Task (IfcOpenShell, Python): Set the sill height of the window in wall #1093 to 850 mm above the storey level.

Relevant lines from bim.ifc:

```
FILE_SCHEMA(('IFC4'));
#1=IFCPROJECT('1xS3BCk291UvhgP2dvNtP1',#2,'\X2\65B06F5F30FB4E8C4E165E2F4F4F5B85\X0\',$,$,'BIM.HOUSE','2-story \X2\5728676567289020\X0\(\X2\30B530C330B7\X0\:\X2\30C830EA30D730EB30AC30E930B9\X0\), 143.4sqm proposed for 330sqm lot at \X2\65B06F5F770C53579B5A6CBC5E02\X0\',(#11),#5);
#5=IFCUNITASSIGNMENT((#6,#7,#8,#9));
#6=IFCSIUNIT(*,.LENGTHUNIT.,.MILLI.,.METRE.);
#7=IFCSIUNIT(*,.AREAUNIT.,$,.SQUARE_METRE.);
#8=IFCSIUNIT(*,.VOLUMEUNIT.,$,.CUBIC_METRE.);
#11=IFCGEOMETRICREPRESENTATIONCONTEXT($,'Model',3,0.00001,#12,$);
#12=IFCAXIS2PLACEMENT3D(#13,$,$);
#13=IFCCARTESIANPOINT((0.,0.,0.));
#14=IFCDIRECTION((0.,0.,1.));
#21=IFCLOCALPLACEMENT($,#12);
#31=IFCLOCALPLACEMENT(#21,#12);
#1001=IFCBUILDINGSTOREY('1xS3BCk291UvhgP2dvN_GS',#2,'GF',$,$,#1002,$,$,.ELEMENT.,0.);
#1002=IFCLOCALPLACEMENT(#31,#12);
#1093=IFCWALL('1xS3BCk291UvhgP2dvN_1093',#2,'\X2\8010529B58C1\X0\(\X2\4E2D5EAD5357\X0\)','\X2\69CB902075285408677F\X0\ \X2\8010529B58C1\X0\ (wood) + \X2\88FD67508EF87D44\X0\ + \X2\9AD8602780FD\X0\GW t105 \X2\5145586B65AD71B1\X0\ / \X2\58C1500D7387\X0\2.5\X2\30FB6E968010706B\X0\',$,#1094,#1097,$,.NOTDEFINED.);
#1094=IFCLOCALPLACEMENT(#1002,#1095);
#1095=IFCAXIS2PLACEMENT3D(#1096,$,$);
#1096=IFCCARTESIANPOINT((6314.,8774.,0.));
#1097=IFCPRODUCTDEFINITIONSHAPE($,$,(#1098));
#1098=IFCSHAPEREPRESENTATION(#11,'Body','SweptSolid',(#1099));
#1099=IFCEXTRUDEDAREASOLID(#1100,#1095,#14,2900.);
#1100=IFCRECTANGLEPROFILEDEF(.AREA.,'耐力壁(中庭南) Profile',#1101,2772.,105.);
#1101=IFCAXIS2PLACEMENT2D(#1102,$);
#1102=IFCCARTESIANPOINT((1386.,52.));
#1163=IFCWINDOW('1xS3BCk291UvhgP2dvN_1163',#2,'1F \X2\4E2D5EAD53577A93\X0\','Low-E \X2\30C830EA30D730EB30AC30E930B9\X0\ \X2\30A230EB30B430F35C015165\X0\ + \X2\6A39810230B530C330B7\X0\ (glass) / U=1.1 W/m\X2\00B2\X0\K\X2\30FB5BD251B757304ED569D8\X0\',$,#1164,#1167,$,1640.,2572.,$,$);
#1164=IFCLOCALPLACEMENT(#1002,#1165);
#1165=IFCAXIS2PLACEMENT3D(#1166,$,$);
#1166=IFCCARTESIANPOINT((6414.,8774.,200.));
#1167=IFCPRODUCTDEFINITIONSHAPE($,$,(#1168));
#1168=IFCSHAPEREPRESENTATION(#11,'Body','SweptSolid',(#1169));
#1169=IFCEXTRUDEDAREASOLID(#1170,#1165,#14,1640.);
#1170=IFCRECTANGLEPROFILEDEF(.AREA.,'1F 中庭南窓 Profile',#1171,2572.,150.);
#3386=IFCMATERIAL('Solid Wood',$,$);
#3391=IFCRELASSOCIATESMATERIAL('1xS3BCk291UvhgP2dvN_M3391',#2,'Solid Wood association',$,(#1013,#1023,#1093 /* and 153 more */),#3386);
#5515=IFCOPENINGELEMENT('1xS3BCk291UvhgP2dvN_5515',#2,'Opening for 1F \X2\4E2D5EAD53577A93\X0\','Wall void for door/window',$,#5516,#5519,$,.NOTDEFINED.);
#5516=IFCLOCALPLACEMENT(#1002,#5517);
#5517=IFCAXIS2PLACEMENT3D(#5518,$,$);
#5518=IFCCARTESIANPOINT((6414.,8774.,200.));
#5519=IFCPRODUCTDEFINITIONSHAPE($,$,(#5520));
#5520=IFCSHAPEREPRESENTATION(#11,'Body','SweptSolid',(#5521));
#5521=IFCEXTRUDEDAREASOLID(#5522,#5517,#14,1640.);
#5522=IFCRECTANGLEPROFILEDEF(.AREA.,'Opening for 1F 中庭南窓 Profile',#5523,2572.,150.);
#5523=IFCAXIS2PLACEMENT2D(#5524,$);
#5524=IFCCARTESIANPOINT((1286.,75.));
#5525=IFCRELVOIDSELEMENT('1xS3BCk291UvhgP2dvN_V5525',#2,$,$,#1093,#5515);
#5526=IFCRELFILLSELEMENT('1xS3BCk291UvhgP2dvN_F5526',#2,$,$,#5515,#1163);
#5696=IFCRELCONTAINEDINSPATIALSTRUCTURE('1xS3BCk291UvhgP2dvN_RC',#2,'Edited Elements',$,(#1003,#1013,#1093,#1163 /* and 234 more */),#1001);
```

```python
import numpy as np
import ifcopenshell
import ifcopenshell.api.geometry
import ifcopenshell.geom
import ifcopenshell.util.element
import ifcopenshell.util.placement
import ifcopenshell.util.shape
import ifcopenshell.util.unit

model = ifcopenshell.open("bim.ifc")
unit_scale = ifcopenshell.util.unit.calculate_unit_scale(model)

window = model.by_id(1163)
opening = window.FillsVoids[0].RelatingOpeningElement
storey = ifcopenshell.util.element.get_container(window, ifc_class="IfcBuildingStorey")
level = ifcopenshell.util.placement.get_local_placement(storey.ObjectPlacement)[2, 3]

# The opening's origin need not be at the sill, so measure its lowest point.
shape = ifcopenshell.geom.create_shape(ifcopenshell.geom.settings(), opening)
bottom = ifcopenshell.util.shape.get_shape_bottom_elevation(shape, shape.geometry) / unit_scale
dz = level + 0.85 / unit_scale - bottom

shift = np.array([0.0, 0.0, dz])
# The window is not placed relative to its opening, so move both.
for product in (opening, window):
    matrix = ifcopenshell.util.placement.get_local_placement(product.ObjectPlacement)
    matrix[:3, 3] += shift
    ifcopenshell.api.geometry.edit_object_placement(model, product=product, matrix=matrix, is_si=False)

print(f"moved by {dz * unit_scale:+.3f} m")

model.write("bim_updated.ifc")
```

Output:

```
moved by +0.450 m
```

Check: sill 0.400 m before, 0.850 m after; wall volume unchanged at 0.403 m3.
